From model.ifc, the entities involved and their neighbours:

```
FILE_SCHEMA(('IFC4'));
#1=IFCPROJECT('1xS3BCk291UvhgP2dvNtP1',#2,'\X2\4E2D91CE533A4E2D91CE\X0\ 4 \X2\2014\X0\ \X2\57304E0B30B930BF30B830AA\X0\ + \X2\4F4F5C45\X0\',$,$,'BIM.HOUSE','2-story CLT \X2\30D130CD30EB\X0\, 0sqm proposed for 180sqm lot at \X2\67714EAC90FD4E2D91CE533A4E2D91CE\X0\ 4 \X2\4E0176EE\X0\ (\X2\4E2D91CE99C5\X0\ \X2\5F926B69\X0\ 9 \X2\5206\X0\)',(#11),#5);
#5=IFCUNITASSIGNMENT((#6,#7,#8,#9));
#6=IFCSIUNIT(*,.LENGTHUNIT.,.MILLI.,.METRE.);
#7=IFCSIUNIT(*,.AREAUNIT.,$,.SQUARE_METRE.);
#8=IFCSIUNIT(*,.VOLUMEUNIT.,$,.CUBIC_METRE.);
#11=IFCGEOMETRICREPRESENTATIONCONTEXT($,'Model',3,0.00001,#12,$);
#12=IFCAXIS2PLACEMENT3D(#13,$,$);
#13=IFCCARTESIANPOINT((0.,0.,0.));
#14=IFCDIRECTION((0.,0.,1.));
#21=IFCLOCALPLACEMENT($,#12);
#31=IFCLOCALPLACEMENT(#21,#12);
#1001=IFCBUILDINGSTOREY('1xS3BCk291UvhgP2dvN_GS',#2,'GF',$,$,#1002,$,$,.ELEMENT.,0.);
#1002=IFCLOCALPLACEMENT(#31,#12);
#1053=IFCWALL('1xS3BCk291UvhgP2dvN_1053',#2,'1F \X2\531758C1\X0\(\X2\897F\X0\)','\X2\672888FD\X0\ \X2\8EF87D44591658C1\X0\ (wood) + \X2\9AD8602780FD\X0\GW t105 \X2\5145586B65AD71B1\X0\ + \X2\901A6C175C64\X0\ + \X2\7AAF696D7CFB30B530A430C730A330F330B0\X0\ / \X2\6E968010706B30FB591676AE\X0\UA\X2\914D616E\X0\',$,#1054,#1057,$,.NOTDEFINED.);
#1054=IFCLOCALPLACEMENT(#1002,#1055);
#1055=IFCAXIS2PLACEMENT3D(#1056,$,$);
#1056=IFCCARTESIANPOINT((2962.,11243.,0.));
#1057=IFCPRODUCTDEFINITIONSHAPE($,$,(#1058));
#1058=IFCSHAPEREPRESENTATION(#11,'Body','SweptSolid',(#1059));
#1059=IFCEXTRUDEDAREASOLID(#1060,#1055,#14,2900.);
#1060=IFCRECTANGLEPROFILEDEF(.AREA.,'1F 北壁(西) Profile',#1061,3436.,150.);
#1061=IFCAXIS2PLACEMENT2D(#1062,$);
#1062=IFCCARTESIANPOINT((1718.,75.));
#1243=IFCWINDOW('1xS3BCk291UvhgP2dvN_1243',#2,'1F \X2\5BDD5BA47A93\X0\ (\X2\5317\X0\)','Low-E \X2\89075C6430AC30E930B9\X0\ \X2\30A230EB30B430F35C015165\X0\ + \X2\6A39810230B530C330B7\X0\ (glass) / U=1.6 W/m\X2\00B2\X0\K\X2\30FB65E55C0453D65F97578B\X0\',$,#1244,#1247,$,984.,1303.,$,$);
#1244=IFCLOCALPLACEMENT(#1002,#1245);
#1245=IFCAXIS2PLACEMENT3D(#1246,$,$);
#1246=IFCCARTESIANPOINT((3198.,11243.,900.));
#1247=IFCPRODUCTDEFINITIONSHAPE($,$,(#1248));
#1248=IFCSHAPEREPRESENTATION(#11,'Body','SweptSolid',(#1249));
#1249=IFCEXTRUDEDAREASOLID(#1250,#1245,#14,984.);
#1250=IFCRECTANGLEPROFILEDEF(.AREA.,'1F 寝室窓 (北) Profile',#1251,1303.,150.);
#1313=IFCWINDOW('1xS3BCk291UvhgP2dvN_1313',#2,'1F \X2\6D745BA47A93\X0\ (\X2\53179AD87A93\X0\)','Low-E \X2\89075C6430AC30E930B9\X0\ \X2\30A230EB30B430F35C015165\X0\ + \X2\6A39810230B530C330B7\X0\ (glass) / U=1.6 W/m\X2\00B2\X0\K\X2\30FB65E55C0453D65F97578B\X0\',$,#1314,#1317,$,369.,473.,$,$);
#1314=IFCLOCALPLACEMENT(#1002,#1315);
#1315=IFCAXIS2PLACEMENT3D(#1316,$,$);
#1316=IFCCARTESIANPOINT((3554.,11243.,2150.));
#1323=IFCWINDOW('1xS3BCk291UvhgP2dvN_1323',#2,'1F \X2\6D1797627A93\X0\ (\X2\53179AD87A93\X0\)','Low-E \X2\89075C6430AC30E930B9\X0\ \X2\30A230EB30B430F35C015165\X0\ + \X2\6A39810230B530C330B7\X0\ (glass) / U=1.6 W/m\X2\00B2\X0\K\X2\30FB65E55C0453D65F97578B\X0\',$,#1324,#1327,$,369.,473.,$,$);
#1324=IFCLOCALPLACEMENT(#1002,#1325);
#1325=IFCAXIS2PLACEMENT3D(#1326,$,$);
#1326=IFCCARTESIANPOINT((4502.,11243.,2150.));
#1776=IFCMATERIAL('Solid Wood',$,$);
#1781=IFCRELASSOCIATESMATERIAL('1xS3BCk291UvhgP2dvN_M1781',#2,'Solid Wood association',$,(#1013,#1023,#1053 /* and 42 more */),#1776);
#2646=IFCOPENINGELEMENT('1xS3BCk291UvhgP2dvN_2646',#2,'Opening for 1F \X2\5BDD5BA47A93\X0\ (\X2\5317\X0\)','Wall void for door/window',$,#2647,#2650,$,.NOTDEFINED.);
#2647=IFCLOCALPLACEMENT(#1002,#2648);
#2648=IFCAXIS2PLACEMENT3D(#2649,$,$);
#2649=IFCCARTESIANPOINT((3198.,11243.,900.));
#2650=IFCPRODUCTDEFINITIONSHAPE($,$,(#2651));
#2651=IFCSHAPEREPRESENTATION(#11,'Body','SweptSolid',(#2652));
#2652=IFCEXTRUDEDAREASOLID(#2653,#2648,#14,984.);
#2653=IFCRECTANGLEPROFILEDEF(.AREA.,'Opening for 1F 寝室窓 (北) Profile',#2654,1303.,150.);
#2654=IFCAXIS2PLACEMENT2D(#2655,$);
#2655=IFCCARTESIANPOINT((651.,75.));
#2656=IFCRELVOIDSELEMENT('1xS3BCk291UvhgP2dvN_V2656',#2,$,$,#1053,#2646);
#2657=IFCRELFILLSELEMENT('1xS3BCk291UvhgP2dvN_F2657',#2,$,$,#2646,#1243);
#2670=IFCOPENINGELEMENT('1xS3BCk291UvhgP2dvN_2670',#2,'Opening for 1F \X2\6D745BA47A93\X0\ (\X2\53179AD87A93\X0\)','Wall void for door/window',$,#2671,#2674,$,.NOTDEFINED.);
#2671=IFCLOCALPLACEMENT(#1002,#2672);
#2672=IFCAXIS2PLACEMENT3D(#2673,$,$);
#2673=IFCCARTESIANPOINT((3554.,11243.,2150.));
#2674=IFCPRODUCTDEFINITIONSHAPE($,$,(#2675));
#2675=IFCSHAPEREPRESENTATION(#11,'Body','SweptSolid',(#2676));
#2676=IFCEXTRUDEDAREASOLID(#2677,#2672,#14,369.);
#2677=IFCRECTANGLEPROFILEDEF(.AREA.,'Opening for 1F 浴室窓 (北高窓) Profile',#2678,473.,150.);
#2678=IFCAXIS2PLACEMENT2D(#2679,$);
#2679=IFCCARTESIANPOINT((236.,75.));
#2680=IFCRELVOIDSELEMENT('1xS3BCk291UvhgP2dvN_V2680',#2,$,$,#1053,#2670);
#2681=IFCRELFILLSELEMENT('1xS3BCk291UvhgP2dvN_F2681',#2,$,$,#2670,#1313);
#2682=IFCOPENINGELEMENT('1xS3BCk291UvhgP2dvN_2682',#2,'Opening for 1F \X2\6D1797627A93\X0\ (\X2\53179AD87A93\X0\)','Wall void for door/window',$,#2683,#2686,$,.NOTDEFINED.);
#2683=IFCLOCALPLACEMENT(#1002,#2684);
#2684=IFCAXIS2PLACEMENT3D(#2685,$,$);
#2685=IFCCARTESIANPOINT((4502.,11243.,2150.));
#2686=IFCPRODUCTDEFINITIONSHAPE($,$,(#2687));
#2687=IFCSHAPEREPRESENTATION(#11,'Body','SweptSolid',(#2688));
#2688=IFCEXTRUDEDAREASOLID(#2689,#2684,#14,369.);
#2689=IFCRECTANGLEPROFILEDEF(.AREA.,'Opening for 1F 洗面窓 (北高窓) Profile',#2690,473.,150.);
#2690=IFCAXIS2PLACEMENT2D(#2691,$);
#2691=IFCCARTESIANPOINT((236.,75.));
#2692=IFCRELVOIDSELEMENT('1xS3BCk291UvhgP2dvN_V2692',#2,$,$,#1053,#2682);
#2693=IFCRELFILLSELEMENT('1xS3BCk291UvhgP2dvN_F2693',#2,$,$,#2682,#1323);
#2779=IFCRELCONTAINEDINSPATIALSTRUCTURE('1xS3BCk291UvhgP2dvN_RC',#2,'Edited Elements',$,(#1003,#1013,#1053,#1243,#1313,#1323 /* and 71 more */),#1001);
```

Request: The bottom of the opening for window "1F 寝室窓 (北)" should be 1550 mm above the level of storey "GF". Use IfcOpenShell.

```python
import numpy as np
import ifcopenshell
import ifcopenshell.api.geometry
import ifcopenshell.geom
import ifcopenshell.util.element
import ifcopenshell.util.placement
import ifcopenshell.util.shape
import ifcopenshell.util.unit

model = ifcopenshell.open("model.ifc")
unit_scale = ifcopenshell.util.unit.calculate_unit_scale(model)

window = model.by_guid("1xS3BCk291UvhgP2dvN_1243")
opening = window.FillsVoids[0].RelatingOpeningElement
storey = ifcopenshell.util.element.get_container(window, ifc_class="IfcBuildingStorey")
level = ifcopenshell.util.placement.get_local_placement(storey.ObjectPlacement)[2, 3]

# The opening's origin need not be at the sill, so measure its lowest point.
shape = ifcopenshell.geom.create_shape(ifcopenshell.geom.settings(), opening)
bottom = ifcopenshell.util.shape.get_shape_bottom_elevation(shape, shape.geometry) / unit_scale
dz = level + 1.55 / unit_scale - bottom

shift = np.array([0.0, 0.0, dz])
# The window is not placed relative to its opening, so move both.
for product in (opening, window):
    matrix = ifcopenshell.util.placement.get_local_placement(product.ObjectPlacement)
    matrix[:3, 3] += shift
    ifcopenshell.api.geometry.edit_object_placement(model, product=product, matrix=matrix, is_si=False)

print(f"moved by {dz * unit_scale:+.3f} m")

model.write("model_updated.ifc")
```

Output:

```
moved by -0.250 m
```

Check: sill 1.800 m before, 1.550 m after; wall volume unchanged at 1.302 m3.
